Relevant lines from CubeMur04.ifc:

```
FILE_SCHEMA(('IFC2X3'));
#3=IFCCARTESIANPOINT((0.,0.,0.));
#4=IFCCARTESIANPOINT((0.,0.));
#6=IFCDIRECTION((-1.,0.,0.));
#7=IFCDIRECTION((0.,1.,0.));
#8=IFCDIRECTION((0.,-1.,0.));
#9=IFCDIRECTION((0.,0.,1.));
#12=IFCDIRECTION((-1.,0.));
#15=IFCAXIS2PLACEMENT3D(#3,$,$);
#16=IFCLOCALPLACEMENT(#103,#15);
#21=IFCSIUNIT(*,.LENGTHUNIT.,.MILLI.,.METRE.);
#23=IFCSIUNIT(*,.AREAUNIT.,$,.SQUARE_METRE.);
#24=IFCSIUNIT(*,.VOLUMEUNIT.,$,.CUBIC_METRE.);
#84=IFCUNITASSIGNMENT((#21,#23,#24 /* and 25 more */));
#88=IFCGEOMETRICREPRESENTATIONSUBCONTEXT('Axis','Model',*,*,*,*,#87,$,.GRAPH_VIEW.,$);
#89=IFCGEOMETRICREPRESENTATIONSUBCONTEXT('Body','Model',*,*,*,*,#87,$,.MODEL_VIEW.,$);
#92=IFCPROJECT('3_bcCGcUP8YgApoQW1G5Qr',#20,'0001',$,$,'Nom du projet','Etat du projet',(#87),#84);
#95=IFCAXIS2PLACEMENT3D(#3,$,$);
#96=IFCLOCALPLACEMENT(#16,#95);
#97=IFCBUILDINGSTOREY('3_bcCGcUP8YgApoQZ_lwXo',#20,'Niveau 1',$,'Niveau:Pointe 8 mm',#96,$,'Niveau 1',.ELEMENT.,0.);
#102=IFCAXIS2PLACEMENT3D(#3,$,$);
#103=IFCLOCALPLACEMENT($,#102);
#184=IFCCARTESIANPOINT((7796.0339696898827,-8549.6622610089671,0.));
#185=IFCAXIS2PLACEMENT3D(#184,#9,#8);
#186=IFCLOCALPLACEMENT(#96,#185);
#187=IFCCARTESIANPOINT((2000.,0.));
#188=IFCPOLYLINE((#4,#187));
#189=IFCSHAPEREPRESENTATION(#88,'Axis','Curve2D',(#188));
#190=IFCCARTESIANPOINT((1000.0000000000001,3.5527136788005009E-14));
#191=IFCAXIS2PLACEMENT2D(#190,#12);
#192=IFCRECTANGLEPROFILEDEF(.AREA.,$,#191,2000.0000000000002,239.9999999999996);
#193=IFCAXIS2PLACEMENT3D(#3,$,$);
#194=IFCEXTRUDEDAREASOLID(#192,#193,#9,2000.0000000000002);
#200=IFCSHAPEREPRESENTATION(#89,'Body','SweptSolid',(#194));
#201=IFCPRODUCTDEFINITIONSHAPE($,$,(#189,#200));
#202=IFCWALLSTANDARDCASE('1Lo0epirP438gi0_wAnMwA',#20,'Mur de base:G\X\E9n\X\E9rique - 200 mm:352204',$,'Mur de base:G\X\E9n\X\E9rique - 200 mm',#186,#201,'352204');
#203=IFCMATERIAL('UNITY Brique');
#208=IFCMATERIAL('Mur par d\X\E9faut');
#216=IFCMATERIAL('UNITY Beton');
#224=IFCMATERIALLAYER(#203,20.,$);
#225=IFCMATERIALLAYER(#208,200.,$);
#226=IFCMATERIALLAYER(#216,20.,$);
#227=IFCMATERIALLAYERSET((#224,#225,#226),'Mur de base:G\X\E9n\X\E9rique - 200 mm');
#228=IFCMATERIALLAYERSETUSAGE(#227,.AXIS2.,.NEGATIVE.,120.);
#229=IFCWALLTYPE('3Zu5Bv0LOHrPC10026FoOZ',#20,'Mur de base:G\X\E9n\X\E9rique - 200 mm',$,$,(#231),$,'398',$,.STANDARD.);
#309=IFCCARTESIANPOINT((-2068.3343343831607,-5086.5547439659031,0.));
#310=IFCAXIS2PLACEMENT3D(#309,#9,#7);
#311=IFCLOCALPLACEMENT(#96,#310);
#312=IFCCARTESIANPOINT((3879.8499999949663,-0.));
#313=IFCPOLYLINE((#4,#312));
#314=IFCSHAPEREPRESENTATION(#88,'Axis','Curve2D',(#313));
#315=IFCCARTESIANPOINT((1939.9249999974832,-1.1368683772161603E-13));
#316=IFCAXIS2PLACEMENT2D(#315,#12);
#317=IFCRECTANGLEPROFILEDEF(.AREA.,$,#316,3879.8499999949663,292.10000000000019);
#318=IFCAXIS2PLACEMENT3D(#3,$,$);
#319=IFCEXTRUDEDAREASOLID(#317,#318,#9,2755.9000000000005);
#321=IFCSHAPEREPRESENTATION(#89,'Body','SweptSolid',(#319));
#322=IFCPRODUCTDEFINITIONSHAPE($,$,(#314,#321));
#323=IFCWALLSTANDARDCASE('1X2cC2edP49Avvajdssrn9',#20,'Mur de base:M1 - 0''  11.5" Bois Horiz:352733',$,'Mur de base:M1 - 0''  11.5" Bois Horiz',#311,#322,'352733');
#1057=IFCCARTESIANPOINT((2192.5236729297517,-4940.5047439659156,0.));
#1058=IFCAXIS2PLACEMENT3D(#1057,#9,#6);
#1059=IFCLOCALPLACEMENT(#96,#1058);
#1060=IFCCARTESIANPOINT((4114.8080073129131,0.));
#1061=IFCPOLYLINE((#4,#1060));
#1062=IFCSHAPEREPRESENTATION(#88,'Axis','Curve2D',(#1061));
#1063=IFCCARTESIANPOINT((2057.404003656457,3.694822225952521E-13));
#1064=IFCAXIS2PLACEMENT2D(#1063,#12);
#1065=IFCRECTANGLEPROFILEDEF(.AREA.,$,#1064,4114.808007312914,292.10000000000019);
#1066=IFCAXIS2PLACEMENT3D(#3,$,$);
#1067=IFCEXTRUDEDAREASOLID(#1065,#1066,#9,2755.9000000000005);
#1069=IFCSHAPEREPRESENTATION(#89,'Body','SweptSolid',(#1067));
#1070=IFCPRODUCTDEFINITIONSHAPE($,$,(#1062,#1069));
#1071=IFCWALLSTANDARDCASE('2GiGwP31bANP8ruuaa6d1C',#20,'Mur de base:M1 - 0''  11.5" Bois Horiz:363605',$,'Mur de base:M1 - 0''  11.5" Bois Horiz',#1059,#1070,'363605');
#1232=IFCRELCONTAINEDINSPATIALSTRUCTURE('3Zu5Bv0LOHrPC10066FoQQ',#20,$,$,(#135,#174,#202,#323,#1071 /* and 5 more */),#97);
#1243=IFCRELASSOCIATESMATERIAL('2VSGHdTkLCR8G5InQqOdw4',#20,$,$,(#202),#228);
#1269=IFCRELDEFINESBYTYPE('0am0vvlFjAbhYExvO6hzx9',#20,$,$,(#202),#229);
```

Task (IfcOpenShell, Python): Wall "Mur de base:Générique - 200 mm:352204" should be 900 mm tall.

```python
import ifcopenshell
import ifcopenshell.geom
import ifcopenshell.util.representation
import ifcopenshell.util.shape
import ifcopenshell.util.unit

model = ifcopenshell.open("CubeMur04.ifc")
unit_scale = ifcopenshell.util.unit.calculate_unit_scale(model)
settings = ifcopenshell.geom.settings()


def volume(element):
    """Net volume in cubic metres, openings subtracted."""
    shape = ifcopenshell.geom.create_shape(settings, element)
    return ifcopenshell.util.shape.get_volume(shape.geometry)


wall = model.by_guid("1Lo0epirP438gi0_wAnMwA")
before = volume(wall)

body = ifcopenshell.util.representation.get_representation(wall, "Model", "Body")
solid = body.Items[0]
old_height = solid.Depth
solid.Depth = 0.9 / unit_scale
after = volume(wall)

print(f"height {old_height:g} -> {solid.Depth:g}, volume {before:.3f} -> {after:.3f} m3")

model.write("CubeMur04_v2.ifc")
```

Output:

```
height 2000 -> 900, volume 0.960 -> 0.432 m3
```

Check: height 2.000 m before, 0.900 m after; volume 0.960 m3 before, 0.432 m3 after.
